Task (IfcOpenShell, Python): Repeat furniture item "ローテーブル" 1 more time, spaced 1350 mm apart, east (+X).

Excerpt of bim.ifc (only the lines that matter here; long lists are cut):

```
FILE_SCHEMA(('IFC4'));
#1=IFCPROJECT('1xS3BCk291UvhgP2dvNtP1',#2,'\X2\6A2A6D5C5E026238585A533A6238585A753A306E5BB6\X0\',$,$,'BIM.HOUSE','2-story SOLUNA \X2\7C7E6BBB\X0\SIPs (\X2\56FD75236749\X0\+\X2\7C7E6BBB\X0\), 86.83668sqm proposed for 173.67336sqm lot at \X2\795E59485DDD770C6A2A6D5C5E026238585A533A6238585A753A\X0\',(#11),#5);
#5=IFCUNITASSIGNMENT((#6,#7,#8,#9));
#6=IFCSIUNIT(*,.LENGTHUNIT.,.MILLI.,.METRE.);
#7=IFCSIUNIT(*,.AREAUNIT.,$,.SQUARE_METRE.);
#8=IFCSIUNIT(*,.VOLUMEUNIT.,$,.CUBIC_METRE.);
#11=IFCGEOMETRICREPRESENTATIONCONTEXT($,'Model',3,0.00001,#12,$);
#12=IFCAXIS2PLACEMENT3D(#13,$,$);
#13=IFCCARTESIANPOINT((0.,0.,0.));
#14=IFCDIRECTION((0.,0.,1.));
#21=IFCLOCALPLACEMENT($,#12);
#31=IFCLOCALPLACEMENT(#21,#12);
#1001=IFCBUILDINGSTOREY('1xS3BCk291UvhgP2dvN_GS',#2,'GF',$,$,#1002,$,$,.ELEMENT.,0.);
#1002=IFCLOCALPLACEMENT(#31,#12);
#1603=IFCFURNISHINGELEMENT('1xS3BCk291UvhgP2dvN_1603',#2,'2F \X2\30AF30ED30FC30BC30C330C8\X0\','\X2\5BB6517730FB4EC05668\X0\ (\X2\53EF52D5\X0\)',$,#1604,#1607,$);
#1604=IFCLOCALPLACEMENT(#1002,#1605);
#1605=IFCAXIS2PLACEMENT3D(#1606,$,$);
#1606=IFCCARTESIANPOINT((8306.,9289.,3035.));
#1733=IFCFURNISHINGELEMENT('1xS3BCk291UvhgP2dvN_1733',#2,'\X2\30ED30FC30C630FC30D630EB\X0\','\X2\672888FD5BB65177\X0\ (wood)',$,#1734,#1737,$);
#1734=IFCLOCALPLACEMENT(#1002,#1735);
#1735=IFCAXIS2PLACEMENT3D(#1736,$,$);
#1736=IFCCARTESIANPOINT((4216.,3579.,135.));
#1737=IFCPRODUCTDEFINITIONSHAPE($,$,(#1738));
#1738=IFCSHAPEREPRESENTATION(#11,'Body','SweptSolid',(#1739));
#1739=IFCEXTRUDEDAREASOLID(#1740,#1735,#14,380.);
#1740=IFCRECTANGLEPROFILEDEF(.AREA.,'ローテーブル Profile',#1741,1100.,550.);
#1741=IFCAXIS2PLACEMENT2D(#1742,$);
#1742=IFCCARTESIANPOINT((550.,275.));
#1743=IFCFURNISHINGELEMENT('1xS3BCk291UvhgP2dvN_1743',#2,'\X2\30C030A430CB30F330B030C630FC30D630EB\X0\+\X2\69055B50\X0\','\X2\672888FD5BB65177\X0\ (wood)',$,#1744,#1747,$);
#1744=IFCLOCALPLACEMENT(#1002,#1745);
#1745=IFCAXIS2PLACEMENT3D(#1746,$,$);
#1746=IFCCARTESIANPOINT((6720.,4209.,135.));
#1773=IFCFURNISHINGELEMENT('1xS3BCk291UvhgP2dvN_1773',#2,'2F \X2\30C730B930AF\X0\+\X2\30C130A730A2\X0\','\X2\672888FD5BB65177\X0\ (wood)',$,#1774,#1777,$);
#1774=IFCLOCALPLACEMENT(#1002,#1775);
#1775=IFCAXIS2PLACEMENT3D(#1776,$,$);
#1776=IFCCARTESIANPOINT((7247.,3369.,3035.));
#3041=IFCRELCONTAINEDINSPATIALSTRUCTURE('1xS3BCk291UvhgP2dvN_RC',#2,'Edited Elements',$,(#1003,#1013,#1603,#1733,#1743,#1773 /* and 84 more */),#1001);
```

```python
import numpy as np
import ifcopenshell
import ifcopenshell.api.geometry
import ifcopenshell.api.root
import ifcopenshell.util.element
import ifcopenshell.util.placement

model = ifcopenshell.open("bim.ifc")


def reuse_history(source, copy):
    """copy_class also copies each property set's owner history, people and application; keep the originals."""
    for rel in copy.IsDefinedBy:
        if rel.is_a("IfcRelDefinesByProperties") and (history := rel.RelatingPropertyDefinition.OwnerHistory):
            rel.RelatingPropertyDefinition.OwnerHistory = source.OwnerHistory
            ifcopenshell.util.element.remove_deep2(model, history)


source = model.by_guid("1xS3BCk291UvhgP2dvN_1733")
base = ifcopenshell.util.placement.get_local_placement(source.ObjectPlacement)
step = np.array([1.0, 0.0, 0.0]) * 1350.0

for i in range(1, 2):
    copy = ifcopenshell.api.root.copy_class(model, product=source)
    copy.Representation = ifcopenshell.util.element.copy_deep(
        model, source.Representation, exclude=["IfcGeometricRepresentationContext", "IfcRepresentationMap"]
    )
    reuse_history(source, copy)
    matrix = base.copy()
    matrix[:3, 3] += i * step
    print("added at", matrix[:3, 3].round(3) + 0.0)
    ifcopenshell.api.geometry.edit_object_placement(model, product=copy, matrix=matrix, is_si=False)

model.write("bim_edited.ifc")
```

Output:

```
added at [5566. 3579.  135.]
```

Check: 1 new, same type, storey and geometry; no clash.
